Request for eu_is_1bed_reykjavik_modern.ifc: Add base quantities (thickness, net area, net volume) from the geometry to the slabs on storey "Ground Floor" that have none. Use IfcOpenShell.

First a look at what the model holds.

```python
import ifcopenshell
import ifcopenshell.util.element
import ifcopenshell.util.unit

model = ifcopenshell.open("eu_is_1bed_reykjavik_modern.ifc")
print(model.schema)
for unit_type in ("LENGTHUNIT", "AREAUNIT", "VOLUMEUNIT"):
    print(unit_type, ifcopenshell.util.unit.calculate_unit_scale(model, unit_type))
storey = next(s for s in model.by_type("IfcBuildingStorey") if s.Name == "Ground Floor")
slabs = [e for e in ifcopenshell.util.element.get_decomposition(storey) if e.is_a("IfcSlab")]
for e in sorted(slabs, key=lambda e: e.id()):
    print(e.id(), e.is_a(), e.Name, list(ifcopenshell.util.element.get_psets(e, qtos_only=True)), sep=" | ")
```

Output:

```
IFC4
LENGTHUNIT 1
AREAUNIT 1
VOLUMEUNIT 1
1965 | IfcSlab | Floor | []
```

```python
import ifcopenshell
import ifcopenshell.api.pset
import ifcopenshell.geom
import ifcopenshell.util.element
import ifcopenshell.util.shape
import ifcopenshell.util.unit

model = ifcopenshell.open("eu_is_1bed_reykjavik_modern.ifc")
unit_scale = ifcopenshell.util.unit.calculate_unit_scale(model)
area_scale = ifcopenshell.util.unit.calculate_unit_scale(model, "AREAUNIT")
volume_scale = ifcopenshell.util.unit.calculate_unit_scale(model, "VOLUMEUNIT")
settings = ifcopenshell.geom.settings()

storey = next(s for s in model.by_type("IfcBuildingStorey") if s.Name == "Ground Floor")
slabs = [e for e in ifcopenshell.util.element.get_decomposition(storey) if e.is_a("IfcSlab")]

for e in sorted(slabs, key=lambda e: e.id()):
    if ifcopenshell.util.element.get_psets(e, qtos_only=True, should_inherit=False):
        continue
    # Geometry comes back in metres, in the element's own axes.
    shape = ifcopenshell.geom.create_shape(settings, e)
    values = {
        "Width": ifcopenshell.util.shape.get_z(shape.geometry) / unit_scale,
        "NetArea": ifcopenshell.util.shape.get_footprint_area(shape.geometry) / area_scale,
        "NetVolume": ifcopenshell.util.shape.get_volume(shape.geometry) / volume_scale,
    }
    qto = ifcopenshell.api.pset.add_qto(model, product=e, name="Qto_SlabBaseQuantities")
    ifcopenshell.api.pset.edit_qto(model, qto=qto, properties=values)
    print(e.id(), {k: round(v, 3) for k, v in values.items()})

model.write("eu_is_1bed_reykjavik_modern-out.ifc")
```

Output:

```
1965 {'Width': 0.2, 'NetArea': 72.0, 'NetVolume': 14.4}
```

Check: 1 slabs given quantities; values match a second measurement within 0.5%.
